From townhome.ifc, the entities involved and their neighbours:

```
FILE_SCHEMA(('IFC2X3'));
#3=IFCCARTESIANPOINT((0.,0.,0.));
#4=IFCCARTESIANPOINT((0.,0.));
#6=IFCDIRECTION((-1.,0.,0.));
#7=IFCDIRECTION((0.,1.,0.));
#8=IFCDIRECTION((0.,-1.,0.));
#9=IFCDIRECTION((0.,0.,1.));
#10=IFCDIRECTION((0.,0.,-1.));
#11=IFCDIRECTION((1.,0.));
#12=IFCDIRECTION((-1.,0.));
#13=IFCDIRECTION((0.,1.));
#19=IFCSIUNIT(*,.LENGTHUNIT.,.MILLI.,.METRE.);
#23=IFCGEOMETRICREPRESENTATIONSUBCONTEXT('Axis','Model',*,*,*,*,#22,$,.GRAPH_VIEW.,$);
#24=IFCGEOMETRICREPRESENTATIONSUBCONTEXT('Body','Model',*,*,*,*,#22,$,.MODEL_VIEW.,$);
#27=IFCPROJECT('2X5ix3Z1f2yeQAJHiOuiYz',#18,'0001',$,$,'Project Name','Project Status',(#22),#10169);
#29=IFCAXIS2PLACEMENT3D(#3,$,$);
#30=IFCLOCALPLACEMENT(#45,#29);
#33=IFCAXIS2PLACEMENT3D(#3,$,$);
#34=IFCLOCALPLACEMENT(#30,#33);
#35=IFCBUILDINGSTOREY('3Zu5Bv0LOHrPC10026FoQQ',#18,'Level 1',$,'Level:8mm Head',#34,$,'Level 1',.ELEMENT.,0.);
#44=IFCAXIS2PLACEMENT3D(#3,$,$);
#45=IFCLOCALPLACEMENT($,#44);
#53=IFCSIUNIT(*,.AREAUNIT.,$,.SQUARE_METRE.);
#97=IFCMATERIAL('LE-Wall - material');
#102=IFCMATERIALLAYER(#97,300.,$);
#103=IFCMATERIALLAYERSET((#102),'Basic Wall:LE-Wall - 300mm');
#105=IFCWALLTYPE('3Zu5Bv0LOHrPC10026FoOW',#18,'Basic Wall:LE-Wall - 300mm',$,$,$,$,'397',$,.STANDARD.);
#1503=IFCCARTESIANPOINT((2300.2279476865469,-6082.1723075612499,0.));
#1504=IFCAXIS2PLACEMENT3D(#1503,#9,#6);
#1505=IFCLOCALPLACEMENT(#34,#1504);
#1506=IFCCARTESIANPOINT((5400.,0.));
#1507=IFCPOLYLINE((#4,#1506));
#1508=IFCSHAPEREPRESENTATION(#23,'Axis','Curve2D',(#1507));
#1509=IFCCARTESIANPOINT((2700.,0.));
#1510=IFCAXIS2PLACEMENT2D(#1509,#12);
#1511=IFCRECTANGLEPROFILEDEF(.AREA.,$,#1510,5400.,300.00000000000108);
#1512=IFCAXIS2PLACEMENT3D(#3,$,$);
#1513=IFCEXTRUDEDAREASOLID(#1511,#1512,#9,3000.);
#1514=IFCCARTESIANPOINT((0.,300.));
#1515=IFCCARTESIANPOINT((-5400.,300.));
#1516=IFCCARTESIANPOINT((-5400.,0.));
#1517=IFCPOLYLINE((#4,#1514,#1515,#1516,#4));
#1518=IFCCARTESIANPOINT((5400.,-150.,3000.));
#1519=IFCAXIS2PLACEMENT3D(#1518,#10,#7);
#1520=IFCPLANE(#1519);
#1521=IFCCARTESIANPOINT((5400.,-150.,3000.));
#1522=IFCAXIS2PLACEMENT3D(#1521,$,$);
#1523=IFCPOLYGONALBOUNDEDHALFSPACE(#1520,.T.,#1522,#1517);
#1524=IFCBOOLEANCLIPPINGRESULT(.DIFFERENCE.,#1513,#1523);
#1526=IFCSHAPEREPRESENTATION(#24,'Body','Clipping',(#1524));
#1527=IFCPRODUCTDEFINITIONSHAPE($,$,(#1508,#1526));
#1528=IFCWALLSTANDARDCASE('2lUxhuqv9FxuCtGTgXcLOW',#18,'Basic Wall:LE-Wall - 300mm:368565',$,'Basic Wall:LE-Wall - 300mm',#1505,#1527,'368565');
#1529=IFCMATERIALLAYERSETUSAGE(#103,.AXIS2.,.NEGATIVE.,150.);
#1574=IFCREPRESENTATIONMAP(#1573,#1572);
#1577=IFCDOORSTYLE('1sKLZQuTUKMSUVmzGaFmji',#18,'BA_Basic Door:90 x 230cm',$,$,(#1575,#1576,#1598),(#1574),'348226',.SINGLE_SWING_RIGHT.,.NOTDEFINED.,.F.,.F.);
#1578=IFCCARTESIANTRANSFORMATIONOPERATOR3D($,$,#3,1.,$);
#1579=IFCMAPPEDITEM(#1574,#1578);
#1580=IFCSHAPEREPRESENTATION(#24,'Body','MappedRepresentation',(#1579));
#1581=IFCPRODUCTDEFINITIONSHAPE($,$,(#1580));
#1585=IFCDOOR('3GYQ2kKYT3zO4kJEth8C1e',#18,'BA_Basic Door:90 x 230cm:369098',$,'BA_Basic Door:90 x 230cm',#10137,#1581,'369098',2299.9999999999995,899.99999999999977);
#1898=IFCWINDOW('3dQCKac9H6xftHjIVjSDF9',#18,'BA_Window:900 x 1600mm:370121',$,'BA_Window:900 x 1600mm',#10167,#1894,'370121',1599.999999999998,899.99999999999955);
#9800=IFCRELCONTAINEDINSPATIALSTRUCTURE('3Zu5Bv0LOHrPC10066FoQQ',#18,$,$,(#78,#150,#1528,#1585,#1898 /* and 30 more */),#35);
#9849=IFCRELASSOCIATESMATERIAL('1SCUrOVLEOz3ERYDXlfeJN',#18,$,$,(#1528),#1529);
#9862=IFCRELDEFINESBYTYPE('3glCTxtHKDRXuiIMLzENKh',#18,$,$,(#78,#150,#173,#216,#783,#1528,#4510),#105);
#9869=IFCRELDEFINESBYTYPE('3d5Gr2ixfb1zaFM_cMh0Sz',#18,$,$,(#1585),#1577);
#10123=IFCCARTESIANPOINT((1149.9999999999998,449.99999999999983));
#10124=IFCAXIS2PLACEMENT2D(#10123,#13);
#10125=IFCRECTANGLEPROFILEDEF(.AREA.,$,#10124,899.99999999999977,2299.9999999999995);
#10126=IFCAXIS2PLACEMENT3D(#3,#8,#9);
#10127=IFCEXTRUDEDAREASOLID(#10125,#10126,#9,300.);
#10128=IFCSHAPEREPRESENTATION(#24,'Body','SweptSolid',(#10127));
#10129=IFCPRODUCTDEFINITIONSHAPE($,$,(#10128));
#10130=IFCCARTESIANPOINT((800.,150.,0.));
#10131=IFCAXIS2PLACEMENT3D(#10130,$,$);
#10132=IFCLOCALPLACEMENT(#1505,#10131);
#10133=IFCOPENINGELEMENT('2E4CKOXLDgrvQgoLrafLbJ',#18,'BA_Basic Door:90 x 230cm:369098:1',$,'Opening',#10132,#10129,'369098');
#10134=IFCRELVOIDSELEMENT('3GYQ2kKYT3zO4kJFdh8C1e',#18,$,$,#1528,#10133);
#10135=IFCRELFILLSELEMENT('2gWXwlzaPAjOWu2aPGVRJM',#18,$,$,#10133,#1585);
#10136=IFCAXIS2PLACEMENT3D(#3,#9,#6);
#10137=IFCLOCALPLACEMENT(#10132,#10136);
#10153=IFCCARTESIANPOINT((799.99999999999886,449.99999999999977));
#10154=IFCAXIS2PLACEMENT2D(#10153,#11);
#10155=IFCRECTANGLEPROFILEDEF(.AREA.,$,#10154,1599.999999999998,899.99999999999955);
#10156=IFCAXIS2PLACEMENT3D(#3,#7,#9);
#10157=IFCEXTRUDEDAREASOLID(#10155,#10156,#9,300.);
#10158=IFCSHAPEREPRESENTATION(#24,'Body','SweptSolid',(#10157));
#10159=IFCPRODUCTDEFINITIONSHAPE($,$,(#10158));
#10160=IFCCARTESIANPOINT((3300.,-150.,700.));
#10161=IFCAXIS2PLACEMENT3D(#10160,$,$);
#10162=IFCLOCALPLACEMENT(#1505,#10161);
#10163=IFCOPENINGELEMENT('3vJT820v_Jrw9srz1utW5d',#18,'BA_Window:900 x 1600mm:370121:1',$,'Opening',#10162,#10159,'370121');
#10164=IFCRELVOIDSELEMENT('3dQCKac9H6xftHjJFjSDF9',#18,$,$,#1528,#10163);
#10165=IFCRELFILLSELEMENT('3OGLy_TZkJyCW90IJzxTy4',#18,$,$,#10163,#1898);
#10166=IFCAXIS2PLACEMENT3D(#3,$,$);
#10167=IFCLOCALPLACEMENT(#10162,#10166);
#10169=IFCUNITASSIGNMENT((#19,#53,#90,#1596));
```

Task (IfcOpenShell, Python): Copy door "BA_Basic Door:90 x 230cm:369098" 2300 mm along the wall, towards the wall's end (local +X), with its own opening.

```python
import ifcopenshell
import ifcopenshell.api.feature
import ifcopenshell.api.geometry
import ifcopenshell.api.root
import ifcopenshell.geom
import ifcopenshell.util.element
import ifcopenshell.util.placement
import ifcopenshell.util.shape
import ifcopenshell.util.unit

model = ifcopenshell.open("townhome.ifc")
unit_scale = ifcopenshell.util.unit.calculate_unit_scale(model)
settings = ifcopenshell.geom.settings()


def volume(element):
    """Net volume in cubic metres, openings subtracted."""
    shape = ifcopenshell.geom.create_shape(settings, element)
    return ifcopenshell.util.shape.get_volume(shape.geometry)


def reuse_history(source, copy):
    """copy_class also copies each property set's owner history, people and application; keep the originals."""
    for rel in copy.IsDefinedBy:
        if rel.is_a("IfcRelDefinesByProperties") and (history := rel.RelatingPropertyDefinition.OwnerHistory):
            rel.RelatingPropertyDefinition.OwnerHistory = source.OwnerHistory
            ifcopenshell.util.element.remove_deep2(model, history)


door = model.by_guid("3GYQ2kKYT3zO4kJEth8C1e")
opening = door.FillsVoids[0].RelatingOpeningElement
wall = opening.VoidsElements[0].RelatingBuildingElement
before = volume(wall)
shift = ifcopenshell.util.placement.get_local_placement(wall.ObjectPlacement)[:3, 0] * 2.3 / unit_scale

# copy_class copies the void relationship, type, container and properties, but no geometry.
new_opening = ifcopenshell.api.root.copy_class(model, product=opening)
new_opening.Representation = ifcopenshell.util.element.copy_deep(
    model, opening.Representation, exclude=["IfcGeometricRepresentationContext", "IfcRepresentationMap"]
)
new_opening.Name = "BA_Basic Door:90 x 230cm"
new_opening.Tag = None
new_door = ifcopenshell.api.root.copy_class(model, product=door)
new_door.Representation = ifcopenshell.util.element.copy_deep(
    model, door.Representation, exclude=["IfcGeometricRepresentationContext", "IfcRepresentationMap"]
)
new_door.Name = "BA_Basic Door:90 x 230cm"
new_door.Tag = None
reuse_history(door, new_door)
fills = ifcopenshell.api.feature.add_filling(model, opening=new_opening, element=new_door)
fills.OwnerHistory = new_door.OwnerHistory  # required in IFC2X3

for old, new in ((opening, new_opening), (door, new_door)):
    matrix = ifcopenshell.util.placement.get_local_placement(old.ObjectPlacement)
    matrix[:3, 3] += shift
    ifcopenshell.api.geometry.edit_object_placement(model, product=new, matrix=matrix, is_si=False)

after = volume(wall)

print(f"wall volume {before:.3f} -> {after:.3f} m3")

model.write("townhome_updated.ifc")
```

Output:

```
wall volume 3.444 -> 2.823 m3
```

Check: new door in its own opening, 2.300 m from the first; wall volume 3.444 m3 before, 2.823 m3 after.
